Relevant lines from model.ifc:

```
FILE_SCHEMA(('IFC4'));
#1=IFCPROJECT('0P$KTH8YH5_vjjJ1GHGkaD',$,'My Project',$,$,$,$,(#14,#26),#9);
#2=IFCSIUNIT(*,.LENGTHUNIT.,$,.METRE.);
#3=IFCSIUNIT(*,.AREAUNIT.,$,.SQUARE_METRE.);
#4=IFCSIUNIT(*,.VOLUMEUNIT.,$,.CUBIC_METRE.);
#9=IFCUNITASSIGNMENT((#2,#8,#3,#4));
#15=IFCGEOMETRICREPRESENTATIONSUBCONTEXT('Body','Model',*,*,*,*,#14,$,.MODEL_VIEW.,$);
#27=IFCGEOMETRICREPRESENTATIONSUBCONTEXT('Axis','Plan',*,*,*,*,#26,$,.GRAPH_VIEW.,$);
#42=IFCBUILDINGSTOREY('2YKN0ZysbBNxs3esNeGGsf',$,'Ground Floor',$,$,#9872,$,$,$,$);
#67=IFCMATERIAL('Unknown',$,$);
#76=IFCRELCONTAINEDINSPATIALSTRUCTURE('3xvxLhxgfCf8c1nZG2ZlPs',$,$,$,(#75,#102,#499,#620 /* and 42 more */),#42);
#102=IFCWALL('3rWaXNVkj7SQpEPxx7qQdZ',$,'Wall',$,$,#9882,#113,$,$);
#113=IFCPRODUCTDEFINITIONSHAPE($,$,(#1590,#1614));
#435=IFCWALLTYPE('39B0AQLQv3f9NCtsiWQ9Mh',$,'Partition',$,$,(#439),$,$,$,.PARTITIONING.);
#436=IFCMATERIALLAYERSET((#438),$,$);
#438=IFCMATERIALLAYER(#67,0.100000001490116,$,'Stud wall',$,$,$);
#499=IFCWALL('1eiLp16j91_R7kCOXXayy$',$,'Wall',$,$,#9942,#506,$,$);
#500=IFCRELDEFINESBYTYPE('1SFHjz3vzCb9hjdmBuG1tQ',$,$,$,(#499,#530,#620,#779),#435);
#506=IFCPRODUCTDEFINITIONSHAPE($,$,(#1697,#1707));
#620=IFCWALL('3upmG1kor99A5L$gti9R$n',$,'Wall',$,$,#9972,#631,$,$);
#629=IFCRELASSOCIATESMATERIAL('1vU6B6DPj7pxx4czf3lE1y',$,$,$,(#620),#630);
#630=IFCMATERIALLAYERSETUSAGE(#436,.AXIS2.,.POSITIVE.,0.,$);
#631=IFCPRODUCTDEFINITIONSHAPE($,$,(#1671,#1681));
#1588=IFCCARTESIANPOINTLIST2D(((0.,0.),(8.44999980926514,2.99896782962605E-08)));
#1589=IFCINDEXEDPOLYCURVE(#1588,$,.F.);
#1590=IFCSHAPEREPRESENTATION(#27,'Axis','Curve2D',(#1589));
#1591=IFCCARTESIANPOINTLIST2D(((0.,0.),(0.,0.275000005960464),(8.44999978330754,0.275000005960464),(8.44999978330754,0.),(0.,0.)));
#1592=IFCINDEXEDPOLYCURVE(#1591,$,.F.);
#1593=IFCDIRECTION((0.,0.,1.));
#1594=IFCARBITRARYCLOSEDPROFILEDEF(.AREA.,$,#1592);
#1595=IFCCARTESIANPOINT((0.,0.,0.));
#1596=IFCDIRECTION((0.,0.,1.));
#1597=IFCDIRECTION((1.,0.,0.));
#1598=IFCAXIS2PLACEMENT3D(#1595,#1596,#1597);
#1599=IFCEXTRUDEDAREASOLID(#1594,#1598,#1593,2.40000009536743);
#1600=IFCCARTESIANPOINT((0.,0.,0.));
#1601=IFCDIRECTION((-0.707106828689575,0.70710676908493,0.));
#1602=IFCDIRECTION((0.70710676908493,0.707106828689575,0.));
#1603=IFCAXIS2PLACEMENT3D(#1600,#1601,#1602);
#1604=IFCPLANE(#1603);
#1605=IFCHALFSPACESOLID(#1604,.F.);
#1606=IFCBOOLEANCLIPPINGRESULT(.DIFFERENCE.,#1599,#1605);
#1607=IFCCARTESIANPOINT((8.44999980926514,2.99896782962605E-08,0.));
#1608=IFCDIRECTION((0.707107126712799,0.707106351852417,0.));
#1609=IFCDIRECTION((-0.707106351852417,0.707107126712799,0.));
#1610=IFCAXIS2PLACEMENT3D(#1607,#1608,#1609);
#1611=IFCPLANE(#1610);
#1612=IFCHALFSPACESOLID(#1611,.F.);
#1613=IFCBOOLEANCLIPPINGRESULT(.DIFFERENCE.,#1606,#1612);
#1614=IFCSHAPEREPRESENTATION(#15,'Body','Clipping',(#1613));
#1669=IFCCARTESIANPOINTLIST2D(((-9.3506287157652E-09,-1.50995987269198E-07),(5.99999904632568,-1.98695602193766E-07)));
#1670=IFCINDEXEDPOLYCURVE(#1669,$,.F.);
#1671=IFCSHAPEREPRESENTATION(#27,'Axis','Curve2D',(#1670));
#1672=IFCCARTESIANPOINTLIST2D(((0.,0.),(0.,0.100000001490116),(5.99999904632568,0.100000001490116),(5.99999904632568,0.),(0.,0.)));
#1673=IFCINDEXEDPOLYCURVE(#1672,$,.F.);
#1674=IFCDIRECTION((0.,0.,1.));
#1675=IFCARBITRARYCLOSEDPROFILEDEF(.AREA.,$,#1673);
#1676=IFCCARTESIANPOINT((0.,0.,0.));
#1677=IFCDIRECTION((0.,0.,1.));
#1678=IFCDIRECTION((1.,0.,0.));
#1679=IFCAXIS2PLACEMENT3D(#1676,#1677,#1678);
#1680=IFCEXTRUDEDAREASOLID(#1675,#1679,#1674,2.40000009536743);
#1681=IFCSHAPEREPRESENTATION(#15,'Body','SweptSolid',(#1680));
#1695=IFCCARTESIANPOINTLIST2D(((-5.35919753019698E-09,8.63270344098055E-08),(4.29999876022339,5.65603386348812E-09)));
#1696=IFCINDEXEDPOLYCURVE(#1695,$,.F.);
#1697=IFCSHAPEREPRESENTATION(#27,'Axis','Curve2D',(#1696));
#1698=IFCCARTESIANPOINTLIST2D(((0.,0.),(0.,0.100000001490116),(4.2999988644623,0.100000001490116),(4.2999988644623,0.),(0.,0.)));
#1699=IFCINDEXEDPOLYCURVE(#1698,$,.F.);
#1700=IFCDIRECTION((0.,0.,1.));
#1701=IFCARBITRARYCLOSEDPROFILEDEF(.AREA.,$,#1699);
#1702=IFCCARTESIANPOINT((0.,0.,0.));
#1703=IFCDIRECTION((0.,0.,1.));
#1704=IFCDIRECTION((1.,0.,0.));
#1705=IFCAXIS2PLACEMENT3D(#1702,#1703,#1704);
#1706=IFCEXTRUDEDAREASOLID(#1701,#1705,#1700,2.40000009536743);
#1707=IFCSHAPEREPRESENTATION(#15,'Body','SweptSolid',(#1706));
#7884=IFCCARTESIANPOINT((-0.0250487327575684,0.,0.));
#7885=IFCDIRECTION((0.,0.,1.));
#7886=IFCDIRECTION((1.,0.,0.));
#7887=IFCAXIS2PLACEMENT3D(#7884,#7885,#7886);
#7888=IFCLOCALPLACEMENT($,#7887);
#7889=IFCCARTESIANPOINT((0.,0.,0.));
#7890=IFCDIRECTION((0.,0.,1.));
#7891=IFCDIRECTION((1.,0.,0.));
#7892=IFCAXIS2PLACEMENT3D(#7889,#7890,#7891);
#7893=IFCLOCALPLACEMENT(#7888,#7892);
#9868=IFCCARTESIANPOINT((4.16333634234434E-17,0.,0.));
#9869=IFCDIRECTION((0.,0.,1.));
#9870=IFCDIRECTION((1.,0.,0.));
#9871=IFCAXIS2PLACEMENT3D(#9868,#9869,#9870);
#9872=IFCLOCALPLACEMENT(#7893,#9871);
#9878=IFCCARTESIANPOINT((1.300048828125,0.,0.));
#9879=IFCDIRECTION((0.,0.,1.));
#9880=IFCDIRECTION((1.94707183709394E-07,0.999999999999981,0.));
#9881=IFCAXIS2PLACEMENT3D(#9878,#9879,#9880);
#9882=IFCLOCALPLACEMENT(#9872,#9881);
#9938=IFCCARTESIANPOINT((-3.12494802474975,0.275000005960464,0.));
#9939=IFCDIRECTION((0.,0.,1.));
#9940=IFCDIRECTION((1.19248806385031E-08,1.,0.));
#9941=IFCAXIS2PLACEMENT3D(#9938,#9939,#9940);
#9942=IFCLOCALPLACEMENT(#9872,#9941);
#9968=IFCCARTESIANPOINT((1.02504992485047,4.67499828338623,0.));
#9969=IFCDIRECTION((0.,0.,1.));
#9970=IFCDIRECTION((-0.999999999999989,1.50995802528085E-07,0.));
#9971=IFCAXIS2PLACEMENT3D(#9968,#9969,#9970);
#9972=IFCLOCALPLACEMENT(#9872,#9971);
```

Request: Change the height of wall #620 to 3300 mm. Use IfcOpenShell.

```python
import ifcopenshell
import ifcopenshell.geom
import ifcopenshell.util.representation
import ifcopenshell.util.shape

model = ifcopenshell.open("model.ifc")
settings = ifcopenshell.geom.settings()


def volume(element):
    """Net volume in cubic metres, openings subtracted."""
    shape = ifcopenshell.geom.create_shape(settings, element)
    return ifcopenshell.util.shape.get_volume(shape.geometry)


wall = model.by_guid("3upmG1kor99A5L$gti9R$n")
before = volume(wall)

body = ifcopenshell.util.representation.get_representation(wall, "Model", "Body")
solid = body.Items[0]
old_height = solid.Depth
solid.Depth = 3.3
after = volume(wall)

print(f"height {old_height:g} -> {solid.Depth:g}, volume {before:.3f} -> {after:.3f} m3")

model.write("model_v2.ifc")
```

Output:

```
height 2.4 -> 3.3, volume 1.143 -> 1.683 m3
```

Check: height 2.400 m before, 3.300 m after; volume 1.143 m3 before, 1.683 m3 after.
